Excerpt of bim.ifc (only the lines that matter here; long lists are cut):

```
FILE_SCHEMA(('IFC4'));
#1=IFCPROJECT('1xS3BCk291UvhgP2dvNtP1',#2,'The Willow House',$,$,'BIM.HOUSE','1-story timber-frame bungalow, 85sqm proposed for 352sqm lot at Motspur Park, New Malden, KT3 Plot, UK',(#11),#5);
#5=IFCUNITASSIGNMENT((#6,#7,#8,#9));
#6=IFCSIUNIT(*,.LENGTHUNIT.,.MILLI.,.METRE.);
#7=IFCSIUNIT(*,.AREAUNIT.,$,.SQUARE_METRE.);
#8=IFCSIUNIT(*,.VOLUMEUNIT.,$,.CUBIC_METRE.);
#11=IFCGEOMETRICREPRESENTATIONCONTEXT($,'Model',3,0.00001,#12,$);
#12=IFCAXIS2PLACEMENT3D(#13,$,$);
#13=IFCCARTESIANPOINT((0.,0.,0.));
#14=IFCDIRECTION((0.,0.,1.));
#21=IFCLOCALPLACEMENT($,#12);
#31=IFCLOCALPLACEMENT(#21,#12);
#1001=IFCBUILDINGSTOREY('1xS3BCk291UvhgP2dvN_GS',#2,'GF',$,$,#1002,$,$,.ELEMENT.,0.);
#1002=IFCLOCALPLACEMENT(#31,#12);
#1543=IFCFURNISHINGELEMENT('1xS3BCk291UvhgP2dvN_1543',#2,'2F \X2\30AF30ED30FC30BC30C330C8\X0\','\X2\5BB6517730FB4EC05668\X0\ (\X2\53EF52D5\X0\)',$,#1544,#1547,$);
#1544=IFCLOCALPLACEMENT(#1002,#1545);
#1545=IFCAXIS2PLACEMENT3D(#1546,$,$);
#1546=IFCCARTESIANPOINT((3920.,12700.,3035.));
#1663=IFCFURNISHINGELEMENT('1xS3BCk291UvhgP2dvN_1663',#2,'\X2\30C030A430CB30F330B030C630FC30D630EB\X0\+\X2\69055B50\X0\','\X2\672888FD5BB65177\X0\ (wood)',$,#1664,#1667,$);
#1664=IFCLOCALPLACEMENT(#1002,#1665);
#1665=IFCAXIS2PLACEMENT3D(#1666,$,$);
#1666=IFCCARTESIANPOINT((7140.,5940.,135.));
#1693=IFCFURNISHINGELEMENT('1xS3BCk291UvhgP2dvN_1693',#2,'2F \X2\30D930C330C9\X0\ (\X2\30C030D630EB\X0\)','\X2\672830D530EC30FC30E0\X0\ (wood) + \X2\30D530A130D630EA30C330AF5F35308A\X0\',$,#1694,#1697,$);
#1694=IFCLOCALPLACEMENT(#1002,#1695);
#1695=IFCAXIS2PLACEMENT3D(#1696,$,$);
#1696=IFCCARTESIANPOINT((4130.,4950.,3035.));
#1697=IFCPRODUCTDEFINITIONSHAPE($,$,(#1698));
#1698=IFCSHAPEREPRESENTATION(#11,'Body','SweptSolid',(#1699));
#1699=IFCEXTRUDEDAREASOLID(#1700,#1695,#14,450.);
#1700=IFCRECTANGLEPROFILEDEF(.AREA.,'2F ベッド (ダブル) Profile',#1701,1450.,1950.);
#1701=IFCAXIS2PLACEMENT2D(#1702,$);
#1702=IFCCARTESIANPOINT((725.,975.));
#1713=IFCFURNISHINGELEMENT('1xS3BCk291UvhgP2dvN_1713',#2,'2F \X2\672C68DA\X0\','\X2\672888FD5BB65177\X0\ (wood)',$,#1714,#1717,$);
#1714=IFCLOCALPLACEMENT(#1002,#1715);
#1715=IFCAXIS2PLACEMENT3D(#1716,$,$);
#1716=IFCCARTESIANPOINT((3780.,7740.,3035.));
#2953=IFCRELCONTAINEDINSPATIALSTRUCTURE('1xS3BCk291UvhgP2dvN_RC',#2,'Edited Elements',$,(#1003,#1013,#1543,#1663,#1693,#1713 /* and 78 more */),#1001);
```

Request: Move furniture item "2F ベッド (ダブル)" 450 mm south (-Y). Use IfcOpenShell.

```python
import ifcopenshell
import ifcopenshell.api.geometry
import ifcopenshell.util.placement

model = ifcopenshell.open("bim.ifc")

item = model.by_id(1693)
matrix = ifcopenshell.util.placement.get_local_placement(item.ObjectPlacement)
matrix[1, 3] -= 450.0
ifcopenshell.api.geometry.edit_object_placement(model, product=item, matrix=matrix, is_si=False)

print(ifcopenshell.util.placement.get_local_placement(item.ObjectPlacement).round(3) + 0.0)

model.write("bim_updated.ifc")
```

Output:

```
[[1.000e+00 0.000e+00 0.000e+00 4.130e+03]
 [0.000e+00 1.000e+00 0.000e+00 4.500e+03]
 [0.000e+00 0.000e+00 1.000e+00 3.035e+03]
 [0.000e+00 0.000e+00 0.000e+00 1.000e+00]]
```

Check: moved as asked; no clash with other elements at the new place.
